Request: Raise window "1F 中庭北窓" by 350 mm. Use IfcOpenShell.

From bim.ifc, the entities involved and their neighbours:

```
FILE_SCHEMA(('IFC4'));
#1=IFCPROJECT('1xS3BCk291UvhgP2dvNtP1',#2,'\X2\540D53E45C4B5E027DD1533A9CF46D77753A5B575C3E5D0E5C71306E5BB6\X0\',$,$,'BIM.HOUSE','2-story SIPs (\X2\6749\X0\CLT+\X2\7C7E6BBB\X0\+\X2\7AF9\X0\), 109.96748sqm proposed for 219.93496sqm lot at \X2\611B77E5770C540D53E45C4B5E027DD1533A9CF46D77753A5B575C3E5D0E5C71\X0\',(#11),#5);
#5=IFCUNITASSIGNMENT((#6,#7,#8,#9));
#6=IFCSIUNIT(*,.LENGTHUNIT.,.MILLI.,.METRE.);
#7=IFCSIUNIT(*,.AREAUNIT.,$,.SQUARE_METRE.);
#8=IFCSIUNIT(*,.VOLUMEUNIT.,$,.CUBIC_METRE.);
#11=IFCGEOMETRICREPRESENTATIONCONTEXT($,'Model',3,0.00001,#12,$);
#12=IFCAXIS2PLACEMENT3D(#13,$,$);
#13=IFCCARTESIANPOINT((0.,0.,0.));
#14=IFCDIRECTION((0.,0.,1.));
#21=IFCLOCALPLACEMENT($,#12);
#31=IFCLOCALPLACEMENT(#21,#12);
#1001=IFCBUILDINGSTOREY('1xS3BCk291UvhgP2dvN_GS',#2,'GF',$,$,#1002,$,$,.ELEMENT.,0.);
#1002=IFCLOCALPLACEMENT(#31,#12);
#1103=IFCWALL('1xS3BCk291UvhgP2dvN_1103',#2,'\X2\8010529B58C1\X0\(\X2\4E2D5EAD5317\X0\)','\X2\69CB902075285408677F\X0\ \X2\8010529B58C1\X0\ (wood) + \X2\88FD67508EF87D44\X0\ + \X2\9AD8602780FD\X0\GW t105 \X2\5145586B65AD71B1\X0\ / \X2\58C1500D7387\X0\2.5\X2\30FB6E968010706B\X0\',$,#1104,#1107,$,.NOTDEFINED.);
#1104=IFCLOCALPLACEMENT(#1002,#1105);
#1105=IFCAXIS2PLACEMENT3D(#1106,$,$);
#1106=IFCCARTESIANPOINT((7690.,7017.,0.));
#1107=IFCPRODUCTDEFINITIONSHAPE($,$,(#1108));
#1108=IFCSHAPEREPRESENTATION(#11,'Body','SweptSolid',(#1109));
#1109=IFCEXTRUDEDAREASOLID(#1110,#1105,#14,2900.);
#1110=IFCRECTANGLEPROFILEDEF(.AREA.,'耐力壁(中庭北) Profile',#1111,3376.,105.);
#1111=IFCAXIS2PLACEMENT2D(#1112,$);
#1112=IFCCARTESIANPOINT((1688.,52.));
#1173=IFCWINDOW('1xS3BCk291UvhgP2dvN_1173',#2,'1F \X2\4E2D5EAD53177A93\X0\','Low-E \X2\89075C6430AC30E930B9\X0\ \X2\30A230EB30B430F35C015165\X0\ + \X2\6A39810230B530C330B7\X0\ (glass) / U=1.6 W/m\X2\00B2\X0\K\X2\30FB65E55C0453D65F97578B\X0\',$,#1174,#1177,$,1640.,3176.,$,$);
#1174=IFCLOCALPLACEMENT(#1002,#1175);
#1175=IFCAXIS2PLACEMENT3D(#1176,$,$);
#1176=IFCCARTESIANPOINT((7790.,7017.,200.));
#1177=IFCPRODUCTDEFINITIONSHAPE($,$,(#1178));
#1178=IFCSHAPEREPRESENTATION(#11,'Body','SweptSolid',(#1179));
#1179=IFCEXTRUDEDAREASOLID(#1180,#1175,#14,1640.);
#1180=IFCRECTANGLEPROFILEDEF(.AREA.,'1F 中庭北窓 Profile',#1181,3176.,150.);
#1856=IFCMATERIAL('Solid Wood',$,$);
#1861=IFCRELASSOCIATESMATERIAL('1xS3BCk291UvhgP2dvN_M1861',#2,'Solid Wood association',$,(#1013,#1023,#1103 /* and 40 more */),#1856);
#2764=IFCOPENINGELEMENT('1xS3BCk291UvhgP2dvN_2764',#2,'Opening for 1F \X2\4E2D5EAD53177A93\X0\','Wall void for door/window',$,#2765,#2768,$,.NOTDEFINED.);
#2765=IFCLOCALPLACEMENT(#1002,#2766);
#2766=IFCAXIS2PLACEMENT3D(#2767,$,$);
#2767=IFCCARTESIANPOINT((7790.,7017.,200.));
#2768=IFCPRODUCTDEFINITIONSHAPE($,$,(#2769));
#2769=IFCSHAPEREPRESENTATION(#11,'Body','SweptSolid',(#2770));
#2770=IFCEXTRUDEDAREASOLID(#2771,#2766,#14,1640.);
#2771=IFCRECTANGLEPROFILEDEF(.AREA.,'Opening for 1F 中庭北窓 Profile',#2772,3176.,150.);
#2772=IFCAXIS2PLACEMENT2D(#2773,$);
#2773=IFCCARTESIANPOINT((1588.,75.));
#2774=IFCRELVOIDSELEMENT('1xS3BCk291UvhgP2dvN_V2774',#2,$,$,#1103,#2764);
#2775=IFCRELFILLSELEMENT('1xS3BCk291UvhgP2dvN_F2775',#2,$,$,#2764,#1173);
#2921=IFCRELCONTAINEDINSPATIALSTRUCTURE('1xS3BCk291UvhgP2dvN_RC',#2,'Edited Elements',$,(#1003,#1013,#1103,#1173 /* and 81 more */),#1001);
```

```python
import numpy as np
import ifcopenshell
import ifcopenshell.api.geometry
import ifcopenshell.util.placement
import ifcopenshell.util.unit

model = ifcopenshell.open("bim.ifc")
unit_scale = ifcopenshell.util.unit.calculate_unit_scale(model)

window = model.by_id(1173)
opening = window.FillsVoids[0].RelatingOpeningElement
dz = 0.35 / unit_scale

shift = np.array([0.0, 0.0, dz])
# The window is not placed relative to its opening, so move both.
for product in (opening, window):
    matrix = ifcopenshell.util.placement.get_local_placement(product.ObjectPlacement)
    matrix[:3, 3] += shift
    ifcopenshell.api.geometry.edit_object_placement(model, product=product, matrix=matrix, is_si=False)

print(f"moved by {dz * unit_scale:+.3f} m")

model.write("bim_edited.ifc")
```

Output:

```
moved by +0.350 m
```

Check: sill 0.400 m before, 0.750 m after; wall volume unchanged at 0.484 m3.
